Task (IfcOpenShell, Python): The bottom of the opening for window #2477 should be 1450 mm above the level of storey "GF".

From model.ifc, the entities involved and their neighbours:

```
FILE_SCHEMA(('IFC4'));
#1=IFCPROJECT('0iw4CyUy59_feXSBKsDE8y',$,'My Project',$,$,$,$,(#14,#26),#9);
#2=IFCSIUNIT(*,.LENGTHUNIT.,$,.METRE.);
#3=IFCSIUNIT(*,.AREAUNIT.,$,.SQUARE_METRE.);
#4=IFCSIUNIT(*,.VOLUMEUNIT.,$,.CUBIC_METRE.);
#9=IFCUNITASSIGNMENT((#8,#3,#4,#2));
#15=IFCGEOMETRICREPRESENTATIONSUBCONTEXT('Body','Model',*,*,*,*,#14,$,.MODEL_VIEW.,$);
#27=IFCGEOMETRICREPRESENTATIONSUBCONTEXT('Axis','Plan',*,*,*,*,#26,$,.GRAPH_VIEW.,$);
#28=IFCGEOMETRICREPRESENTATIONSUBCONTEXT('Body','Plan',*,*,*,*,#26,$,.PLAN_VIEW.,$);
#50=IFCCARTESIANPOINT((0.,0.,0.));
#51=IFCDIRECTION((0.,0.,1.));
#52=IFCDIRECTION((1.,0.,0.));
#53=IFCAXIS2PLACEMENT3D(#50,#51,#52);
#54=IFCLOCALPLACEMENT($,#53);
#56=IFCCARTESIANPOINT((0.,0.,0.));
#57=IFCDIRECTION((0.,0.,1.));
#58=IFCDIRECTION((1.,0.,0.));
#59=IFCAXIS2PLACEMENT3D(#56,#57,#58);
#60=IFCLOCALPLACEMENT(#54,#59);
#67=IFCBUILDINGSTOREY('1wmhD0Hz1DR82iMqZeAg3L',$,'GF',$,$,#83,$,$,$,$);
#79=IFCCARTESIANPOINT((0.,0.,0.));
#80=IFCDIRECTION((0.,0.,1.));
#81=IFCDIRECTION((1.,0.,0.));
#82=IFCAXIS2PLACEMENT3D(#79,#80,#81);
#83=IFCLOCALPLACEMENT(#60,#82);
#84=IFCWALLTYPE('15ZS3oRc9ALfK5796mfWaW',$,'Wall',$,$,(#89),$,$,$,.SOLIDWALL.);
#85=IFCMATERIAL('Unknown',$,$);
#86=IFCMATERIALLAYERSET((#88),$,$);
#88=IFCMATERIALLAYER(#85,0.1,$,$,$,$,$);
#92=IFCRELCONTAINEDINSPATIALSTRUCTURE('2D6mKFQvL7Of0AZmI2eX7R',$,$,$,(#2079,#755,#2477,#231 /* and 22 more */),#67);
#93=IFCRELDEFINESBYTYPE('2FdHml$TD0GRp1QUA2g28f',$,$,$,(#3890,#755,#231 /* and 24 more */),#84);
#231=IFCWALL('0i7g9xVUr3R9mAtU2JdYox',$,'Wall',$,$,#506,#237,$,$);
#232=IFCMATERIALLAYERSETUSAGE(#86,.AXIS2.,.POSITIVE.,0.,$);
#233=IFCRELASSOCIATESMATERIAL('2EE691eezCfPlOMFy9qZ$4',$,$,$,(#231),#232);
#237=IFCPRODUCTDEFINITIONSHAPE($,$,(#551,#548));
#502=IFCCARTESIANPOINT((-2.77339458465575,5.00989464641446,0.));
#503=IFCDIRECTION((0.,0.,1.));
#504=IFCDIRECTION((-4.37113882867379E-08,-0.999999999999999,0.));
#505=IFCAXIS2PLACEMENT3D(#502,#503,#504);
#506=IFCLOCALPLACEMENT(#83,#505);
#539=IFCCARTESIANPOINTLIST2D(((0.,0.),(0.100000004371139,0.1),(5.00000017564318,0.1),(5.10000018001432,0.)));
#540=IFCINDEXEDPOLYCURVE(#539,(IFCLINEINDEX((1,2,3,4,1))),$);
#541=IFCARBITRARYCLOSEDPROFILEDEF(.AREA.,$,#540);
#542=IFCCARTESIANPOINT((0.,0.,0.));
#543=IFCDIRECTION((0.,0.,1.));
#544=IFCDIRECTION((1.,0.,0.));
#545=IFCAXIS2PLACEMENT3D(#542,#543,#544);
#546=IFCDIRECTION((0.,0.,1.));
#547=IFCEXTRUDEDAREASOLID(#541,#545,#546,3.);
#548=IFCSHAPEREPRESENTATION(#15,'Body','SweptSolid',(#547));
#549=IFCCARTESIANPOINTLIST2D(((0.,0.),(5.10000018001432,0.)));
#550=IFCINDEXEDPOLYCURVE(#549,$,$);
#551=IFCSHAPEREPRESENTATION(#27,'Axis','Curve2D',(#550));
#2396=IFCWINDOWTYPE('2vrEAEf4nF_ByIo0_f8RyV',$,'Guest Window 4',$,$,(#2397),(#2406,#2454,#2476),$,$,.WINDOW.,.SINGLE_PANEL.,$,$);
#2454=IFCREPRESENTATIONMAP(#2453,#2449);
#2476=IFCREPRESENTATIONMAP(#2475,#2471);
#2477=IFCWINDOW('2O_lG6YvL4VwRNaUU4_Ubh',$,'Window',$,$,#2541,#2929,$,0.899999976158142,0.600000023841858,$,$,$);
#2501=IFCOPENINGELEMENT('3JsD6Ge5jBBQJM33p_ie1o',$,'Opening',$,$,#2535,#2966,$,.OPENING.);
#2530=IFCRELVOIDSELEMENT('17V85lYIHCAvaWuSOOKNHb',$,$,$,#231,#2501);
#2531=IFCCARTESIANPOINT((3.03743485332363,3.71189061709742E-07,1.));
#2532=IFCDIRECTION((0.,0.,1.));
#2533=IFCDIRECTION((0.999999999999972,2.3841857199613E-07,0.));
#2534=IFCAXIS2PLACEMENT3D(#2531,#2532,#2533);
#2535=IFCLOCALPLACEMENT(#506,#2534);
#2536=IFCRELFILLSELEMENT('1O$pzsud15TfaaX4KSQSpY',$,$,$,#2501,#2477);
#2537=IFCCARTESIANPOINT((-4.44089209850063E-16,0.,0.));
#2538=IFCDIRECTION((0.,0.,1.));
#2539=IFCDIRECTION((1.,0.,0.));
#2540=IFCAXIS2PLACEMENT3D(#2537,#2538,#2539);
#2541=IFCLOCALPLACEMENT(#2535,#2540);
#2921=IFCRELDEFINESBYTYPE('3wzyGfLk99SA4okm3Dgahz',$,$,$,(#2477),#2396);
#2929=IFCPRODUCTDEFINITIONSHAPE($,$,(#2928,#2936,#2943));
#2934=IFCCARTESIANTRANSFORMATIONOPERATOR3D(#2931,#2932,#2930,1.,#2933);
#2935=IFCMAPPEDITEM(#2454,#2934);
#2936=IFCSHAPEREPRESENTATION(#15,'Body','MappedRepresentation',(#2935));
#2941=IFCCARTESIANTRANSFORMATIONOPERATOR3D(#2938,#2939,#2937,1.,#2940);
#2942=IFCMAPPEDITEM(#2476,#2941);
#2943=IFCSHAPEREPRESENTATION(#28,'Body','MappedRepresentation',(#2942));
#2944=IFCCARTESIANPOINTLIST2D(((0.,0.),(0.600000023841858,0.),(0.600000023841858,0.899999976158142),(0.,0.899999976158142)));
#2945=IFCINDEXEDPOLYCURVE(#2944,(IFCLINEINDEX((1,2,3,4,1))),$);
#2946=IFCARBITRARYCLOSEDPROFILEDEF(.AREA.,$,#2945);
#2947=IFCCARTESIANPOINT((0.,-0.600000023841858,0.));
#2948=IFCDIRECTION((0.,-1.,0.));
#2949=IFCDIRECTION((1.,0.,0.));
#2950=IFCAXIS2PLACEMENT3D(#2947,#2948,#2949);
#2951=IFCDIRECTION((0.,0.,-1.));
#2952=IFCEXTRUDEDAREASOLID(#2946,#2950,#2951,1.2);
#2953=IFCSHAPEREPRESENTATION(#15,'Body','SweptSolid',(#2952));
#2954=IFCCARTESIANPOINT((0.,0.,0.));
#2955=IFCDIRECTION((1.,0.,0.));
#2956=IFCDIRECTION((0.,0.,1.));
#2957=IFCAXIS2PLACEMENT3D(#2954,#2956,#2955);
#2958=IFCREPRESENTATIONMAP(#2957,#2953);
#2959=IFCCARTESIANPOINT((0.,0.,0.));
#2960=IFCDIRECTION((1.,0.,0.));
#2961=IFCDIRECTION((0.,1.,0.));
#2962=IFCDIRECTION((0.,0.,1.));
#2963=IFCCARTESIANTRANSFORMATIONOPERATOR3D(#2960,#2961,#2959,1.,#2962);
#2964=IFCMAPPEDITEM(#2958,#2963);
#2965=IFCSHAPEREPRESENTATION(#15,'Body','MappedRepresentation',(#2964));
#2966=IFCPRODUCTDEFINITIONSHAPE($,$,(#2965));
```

```python
import numpy as np
import ifcopenshell
import ifcopenshell.api.geometry
import ifcopenshell.geom
import ifcopenshell.util.element
import ifcopenshell.util.placement
import ifcopenshell.util.shape
import ifcopenshell.util.unit

model = ifcopenshell.open("model.ifc")
unit_scale = ifcopenshell.util.unit.calculate_unit_scale(model)

window = model.by_guid("2O_lG6YvL4VwRNaUU4_Ubh")
opening = window.FillsVoids[0].RelatingOpeningElement
storey = ifcopenshell.util.element.get_container(window, ifc_class="IfcBuildingStorey")
level = ifcopenshell.util.placement.get_local_placement(storey.ObjectPlacement)[2, 3]

# The opening's origin need not be at the sill, so measure its lowest point.
shape = ifcopenshell.geom.create_shape(ifcopenshell.geom.settings(), opening)
bottom = ifcopenshell.util.shape.get_shape_bottom_elevation(shape, shape.geometry) / unit_scale
dz = level + 1.45 / unit_scale - bottom

shift = np.array([0.0, 0.0, dz])
# The window is placed relative to its opening, so it follows when the opening moves.
matrix = ifcopenshell.util.placement.get_local_placement(opening.ObjectPlacement)
matrix[:3, 3] += shift
ifcopenshell.api.geometry.edit_object_placement(
    model, product=opening, matrix=matrix, is_si=False, should_transform_children=True
)

print(f"moved by {dz * unit_scale:+.3f} m")

model.write("model-out.ifc")
```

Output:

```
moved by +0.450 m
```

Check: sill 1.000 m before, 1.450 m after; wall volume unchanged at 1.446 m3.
